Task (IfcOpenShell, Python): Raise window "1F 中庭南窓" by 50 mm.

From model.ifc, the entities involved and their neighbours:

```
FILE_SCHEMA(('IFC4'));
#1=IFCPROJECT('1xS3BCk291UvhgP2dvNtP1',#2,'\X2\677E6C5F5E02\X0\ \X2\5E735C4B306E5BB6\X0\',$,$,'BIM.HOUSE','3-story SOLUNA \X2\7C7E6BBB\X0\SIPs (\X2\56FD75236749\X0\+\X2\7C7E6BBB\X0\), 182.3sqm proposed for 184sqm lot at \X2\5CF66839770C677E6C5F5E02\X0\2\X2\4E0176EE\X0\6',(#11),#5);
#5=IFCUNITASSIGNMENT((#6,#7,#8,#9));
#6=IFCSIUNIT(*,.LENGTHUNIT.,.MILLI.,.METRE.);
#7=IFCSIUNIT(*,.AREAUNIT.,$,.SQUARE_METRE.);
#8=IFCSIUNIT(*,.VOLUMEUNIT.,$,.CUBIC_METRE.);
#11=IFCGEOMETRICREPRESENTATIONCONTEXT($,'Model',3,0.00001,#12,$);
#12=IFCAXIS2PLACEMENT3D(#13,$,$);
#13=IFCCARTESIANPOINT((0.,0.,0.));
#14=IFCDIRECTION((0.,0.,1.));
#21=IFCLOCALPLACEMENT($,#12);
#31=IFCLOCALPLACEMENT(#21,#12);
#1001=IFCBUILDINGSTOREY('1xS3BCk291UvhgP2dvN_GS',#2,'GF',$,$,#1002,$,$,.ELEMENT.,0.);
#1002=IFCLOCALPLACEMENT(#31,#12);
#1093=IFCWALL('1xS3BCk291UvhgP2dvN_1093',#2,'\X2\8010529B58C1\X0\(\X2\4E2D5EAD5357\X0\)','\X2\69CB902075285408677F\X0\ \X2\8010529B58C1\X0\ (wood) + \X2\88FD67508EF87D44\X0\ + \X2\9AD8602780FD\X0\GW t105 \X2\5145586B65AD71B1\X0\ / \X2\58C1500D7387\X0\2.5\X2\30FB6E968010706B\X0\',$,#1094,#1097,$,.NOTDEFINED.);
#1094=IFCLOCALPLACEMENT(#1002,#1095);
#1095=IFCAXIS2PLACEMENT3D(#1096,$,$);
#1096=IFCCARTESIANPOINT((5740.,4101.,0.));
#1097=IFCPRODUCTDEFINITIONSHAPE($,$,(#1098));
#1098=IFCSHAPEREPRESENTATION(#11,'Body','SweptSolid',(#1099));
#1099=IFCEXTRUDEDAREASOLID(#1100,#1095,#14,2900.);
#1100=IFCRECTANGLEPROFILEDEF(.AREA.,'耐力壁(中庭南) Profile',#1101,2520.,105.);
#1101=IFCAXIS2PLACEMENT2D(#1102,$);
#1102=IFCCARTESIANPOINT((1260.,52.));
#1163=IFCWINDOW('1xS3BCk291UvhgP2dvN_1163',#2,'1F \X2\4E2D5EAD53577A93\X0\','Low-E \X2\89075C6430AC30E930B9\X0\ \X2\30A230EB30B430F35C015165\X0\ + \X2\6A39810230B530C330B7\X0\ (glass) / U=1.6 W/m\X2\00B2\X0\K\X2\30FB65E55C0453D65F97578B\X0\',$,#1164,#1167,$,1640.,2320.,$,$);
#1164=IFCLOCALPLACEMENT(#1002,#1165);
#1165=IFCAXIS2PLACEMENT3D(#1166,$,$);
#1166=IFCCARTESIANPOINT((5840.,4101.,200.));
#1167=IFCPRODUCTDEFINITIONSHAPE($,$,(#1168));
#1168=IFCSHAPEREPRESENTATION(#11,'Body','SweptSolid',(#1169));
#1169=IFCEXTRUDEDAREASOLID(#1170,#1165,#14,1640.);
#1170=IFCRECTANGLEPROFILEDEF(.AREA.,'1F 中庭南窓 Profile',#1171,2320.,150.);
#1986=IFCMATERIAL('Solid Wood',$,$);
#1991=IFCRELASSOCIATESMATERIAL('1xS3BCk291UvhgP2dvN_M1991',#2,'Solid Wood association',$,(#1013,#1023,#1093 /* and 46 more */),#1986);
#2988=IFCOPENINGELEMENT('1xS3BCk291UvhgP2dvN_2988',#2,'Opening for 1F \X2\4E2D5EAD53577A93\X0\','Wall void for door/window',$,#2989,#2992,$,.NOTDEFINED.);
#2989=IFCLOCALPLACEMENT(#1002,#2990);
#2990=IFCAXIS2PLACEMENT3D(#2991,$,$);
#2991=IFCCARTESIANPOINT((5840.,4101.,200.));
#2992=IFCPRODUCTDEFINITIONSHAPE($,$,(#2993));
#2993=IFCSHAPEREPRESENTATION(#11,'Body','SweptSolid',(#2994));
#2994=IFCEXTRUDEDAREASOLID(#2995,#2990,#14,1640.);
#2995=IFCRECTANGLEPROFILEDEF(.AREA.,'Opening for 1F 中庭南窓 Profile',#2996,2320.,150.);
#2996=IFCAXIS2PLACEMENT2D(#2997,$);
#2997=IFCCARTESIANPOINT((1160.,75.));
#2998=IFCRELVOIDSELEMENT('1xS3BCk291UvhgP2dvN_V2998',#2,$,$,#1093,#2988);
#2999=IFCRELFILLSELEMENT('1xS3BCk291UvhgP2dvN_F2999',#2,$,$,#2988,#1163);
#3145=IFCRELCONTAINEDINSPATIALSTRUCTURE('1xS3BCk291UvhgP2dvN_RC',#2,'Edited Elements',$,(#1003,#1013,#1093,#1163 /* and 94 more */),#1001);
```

```python
import numpy as np
import ifcopenshell
import ifcopenshell.api.geometry
import ifcopenshell.util.placement
import ifcopenshell.util.unit

model = ifcopenshell.open("model.ifc")
unit_scale = ifcopenshell.util.unit.calculate_unit_scale(model)

window = model.by_guid("1xS3BCk291UvhgP2dvN_1163")
opening = window.FillsVoids[0].RelatingOpeningElement
dz = 0.05 / unit_scale

shift = np.array([0.0, 0.0, dz])
# The window is not placed relative to its opening, so move both.
for product in (opening, window):
    matrix = ifcopenshell.util.placement.get_local_placement(product.ObjectPlacement)
    matrix[:3, 3] += shift
    ifcopenshell.api.geometry.edit_object_placement(model, product=product, matrix=matrix, is_si=False)

print(f"moved by {dz * unit_scale:+.3f} m")

model.write("model_v2.ifc")
```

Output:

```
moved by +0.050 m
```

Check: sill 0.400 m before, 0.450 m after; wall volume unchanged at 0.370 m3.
